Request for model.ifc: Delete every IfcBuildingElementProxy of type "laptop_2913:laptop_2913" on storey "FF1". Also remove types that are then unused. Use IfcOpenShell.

First a look at what the model holds.

```python
import ifcopenshell
import ifcopenshell.util.element

model = ifcopenshell.open("model.ifc")
print(model.schema)
storey = next(s for s in model.by_type("IfcBuildingStorey") if s.Name == "FF1")
proxies = [e for e in ifcopenshell.util.element.get_decomposition(storey) if e.is_a("IfcBuildingElementProxy")]
seen = {}
for e in proxies:
    element_type = ifcopenshell.util.element.get_type(e)
    name = element_type.Name if element_type not in (None, e) else None
    seen[name] = seen.get(name, 0) + 1
for name, count in sorted(seen.items(), key=str):
    print(count, "x", name)
```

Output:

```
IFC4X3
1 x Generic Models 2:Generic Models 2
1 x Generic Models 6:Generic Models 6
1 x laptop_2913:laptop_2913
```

```python
import ifcopenshell
import ifcopenshell.api.root
import ifcopenshell.util.element

model = ifcopenshell.open("model.ifc")

storey = next(s for s in model.by_type("IfcBuildingStorey") if s.Name == "FF1")
proxies = [e for e in ifcopenshell.util.element.get_decomposition(storey) if e.is_a("IfcBuildingElementProxy")]
targets = [e for e in proxies if (t := ifcopenshell.util.element.get_type(e)) not in (None, e) and t.Name == "laptop_2913:laptop_2913"]
types = {ifcopenshell.util.element.get_type(e) for e in targets} - {None, *targets}

for e in targets:
    ifcopenshell.api.root.remove_product(model, product=e)
print(len(targets), "removed")

unused = [t for t in types if not ifcopenshell.util.element.get_types(t)]
for t in unused:
    ifcopenshell.api.root.remove_product(model, product=t)
print(len(unused), "unused types removed")

model.write("model_rev.ifc")
```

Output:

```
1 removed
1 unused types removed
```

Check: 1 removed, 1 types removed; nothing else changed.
